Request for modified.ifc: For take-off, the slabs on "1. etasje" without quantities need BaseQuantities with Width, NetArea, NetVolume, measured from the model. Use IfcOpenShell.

First a look at what the model holds.

```python
import ifcopenshell
import ifcopenshell.util.element
import ifcopenshell.util.unit

model = ifcopenshell.open("modified.ifc")
print(model.schema)
for unit_type in ("LENGTHUNIT", "AREAUNIT", "VOLUMEUNIT"):
    print(unit_type, ifcopenshell.util.unit.calculate_unit_scale(model, unit_type))
storey = next(s for s in model.by_type("IfcBuildingStorey") if s.Name == "1. etasje")
slabs = [e for e in ifcopenshell.util.element.get_decomposition(storey) if e.is_a("IfcSlab")]
for e in sorted(slabs, key=lambda e: e.id()):
    print(e.id(), e.is_a(), e.Name, list(ifcopenshell.util.element.get_psets(e, qtos_only=True)), sep=" | ")
```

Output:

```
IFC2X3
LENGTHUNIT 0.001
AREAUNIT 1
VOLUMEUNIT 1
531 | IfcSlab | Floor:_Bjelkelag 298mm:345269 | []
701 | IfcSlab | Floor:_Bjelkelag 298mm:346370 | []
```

```python
import ifcopenshell
import ifcopenshell.api.pset
import ifcopenshell.geom
import ifcopenshell.util.element
import ifcopenshell.util.shape
import ifcopenshell.util.unit

model = ifcopenshell.open("modified.ifc")
unit_scale = ifcopenshell.util.unit.calculate_unit_scale(model)
area_scale = ifcopenshell.util.unit.calculate_unit_scale(model, "AREAUNIT")
volume_scale = ifcopenshell.util.unit.calculate_unit_scale(model, "VOLUMEUNIT")
settings = ifcopenshell.geom.settings()

storey = next(s for s in model.by_type("IfcBuildingStorey") if s.Name == "1. etasje")
slabs = [e for e in ifcopenshell.util.element.get_decomposition(storey) if e.is_a("IfcSlab")]

for e in sorted(slabs, key=lambda e: e.id()):
    if ifcopenshell.util.element.get_psets(e, qtos_only=True, should_inherit=False):
        continue
    # Geometry comes back in metres, in the element's own axes.
    shape = ifcopenshell.geom.create_shape(settings, e)
    values = {
        "Width": ifcopenshell.util.shape.get_z(shape.geometry) / unit_scale,
        "NetArea": ifcopenshell.util.shape.get_footprint_area(shape.geometry) / area_scale,
        "NetVolume": ifcopenshell.util.shape.get_volume(shape.geometry) / volume_scale,
    }
    qto = ifcopenshell.api.pset.add_qto(model, product=e, name="BaseQuantities")
    ifcopenshell.api.pset.edit_qto(model, qto=qto, properties=values)
    print(e.id(), {k: round(v, 3) for k, v in values.items()})

model.write("modified_v2.ifc")
```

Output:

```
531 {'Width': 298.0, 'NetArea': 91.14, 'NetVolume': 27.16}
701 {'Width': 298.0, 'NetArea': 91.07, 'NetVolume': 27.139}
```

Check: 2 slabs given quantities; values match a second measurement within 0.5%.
